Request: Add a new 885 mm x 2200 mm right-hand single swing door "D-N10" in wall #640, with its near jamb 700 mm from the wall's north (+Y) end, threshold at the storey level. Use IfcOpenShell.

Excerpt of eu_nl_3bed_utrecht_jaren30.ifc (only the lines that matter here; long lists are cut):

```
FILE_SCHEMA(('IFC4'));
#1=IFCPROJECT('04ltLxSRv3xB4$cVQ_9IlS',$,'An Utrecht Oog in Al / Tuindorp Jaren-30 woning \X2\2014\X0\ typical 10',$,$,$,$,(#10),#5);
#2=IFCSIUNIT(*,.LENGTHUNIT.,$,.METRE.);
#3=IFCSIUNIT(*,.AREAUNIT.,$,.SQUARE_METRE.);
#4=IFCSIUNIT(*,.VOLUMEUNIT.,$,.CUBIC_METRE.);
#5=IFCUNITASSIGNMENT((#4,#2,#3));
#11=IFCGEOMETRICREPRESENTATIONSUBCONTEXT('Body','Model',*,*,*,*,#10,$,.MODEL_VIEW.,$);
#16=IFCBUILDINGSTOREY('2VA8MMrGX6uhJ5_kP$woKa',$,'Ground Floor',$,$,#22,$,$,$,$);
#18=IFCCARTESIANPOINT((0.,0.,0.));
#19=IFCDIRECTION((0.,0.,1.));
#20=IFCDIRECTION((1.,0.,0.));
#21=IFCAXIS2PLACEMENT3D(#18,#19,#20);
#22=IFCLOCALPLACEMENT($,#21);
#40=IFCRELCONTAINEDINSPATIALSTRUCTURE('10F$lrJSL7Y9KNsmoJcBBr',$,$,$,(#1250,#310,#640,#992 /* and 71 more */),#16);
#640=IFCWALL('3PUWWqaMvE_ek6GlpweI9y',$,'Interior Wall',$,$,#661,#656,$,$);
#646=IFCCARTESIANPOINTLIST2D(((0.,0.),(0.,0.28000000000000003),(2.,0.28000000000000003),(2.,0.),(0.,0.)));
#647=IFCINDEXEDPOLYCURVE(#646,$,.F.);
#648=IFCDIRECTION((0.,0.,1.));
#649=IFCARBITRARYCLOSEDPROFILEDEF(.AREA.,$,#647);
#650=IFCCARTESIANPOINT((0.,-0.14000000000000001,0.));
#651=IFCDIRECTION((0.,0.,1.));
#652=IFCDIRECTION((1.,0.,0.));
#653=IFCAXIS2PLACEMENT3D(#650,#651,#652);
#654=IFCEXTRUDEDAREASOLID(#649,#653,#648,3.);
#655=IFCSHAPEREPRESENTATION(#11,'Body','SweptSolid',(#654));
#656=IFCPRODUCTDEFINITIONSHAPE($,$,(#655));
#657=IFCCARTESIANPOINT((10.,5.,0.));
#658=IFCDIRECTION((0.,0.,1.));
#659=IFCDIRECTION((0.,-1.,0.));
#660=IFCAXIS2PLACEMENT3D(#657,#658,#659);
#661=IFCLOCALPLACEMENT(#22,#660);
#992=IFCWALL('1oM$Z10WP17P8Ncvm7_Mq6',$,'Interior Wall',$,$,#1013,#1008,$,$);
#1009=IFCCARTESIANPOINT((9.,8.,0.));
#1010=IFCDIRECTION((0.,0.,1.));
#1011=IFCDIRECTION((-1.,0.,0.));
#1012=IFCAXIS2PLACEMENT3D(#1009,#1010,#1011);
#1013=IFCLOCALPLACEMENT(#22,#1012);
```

```python
import numpy as np
import ifcopenshell
import ifcopenshell.api.feature
import ifcopenshell.api.geometry
import ifcopenshell.api.root
import ifcopenshell.api.spatial
import ifcopenshell.geom
import ifcopenshell.util.element
import ifcopenshell.util.placement
import ifcopenshell.util.representation
import ifcopenshell.util.shape
import ifcopenshell.util.unit

model = ifcopenshell.open("eu_nl_3bed_utrecht_jaren30.ifc")
unit_scale = ifcopenshell.util.unit.calculate_unit_scale(model)
settings = ifcopenshell.geom.settings()


def volume(element):
    """Net volume in cubic metres, openings subtracted."""
    shape = ifcopenshell.geom.create_shape(settings, element)
    return ifcopenshell.util.shape.get_volume(shape.geometry)


wall = model.by_guid("3PUWWqaMvE_ek6GlpweI9y")
storey = ifcopenshell.util.element.get_container(wall, ifc_class="IfcBuildingStorey")
context = ifcopenshell.util.representation.get_context(model, "Model", "Body", "MODEL_VIEW")
before = volume(wall)

width, height, from_end, sill = 0.885, 2.2, 0.7, 0.0  # metres

# The wall runs along its own X axis, and the end named is its -X end.
wall_shape = ifcopenshell.geom.create_shape(settings, wall)
x, y, z = ifcopenshell.util.shape.get_vertices(wall_shape.geometry).T
start = x.min() + from_end
face, thickness = float(y.min()), float(y.max() - y.min())
wall_matrix = ifcopenshell.util.placement.get_local_placement(wall.ObjectPlacement)
level = ifcopenshell.util.placement.get_local_placement(storey.ObjectPlacement)[2, 3]


def in_wall(x, y):
    """Placement at x, y metres in the wall's axes, at sill height."""
    matrix = wall_matrix.copy()
    matrix[:, 3] = wall_matrix @ np.array([x / unit_scale, y / unit_scale, 0.0, 1.0])
    matrix[2, 3] = level + sill / unit_scale
    return matrix


# Opening: a box that overshoots both wall faces by 50 mm.
opening = ifcopenshell.api.root.create_entity(model, ifc_class="IfcOpeningElement", predefined_type="OPENING")
box = ifcopenshell.api.geometry.add_wall_representation(
    model, context=context, length=width, height=height, thickness=thickness + 0.1
)
ifcopenshell.api.geometry.assign_representation(model, product=opening, representation=box)
ifcopenshell.api.geometry.edit_object_placement(model, product=opening, matrix=in_wall(start, face - 0.05), is_si=False)
ifcopenshell.api.feature.add_feature(model, feature=opening, element=wall)

door = ifcopenshell.api.root.create_entity(model, ifc_class="IfcDoor", name="D-N10", predefined_type="DOOR")
door.OverallWidth, door.OverallHeight = width / unit_scale, height / unit_scale
door.OperationType = "SINGLE_SWING_RIGHT"
body = ifcopenshell.api.geometry.add_door_representation(
    model,
    context=context,
    overall_width=door.OverallWidth,
    overall_height=door.OverallHeight,
    operation_type="SINGLE_SWING_RIGHT",
    lining_properties={"LiningDepth": thickness / unit_scale, "ThresholdDepth": thickness / unit_scale},
)
ifcopenshell.api.geometry.assign_representation(model, product=door, representation=body)
ifcopenshell.api.spatial.assign_container(model, products=[door], relating_structure=storey)
ifcopenshell.api.feature.add_filling(model, opening=opening, element=door)

# The lining spans the wall, so the door starts at the wall face.
ifcopenshell.api.geometry.edit_object_placement(model, product=door, matrix=in_wall(start, face), is_si=False)

after = volume(wall)

print(f"wall volume {before:.3f} -> {after:.3f} m3")

model.write("eu_nl_3bed_utrecht_jaren30_updated.ifc")
```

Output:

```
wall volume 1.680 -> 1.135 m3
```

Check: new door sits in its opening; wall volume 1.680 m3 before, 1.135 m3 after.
